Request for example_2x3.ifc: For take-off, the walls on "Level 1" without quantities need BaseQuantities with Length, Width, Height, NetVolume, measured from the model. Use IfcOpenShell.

First a look at what the model holds.

```python
import ifcopenshell
import ifcopenshell.util.element
import ifcopenshell.util.unit

model = ifcopenshell.open("example_2x3.ifc")
print(model.schema)
for unit_type in ("LENGTHUNIT", "AREAUNIT", "VOLUMEUNIT"):
    print(unit_type, ifcopenshell.util.unit.calculate_unit_scale(model, unit_type))
storey = next(s for s in model.by_type("IfcBuildingStorey") if s.Name == "Level 1")
walls = [e for e in ifcopenshell.util.element.get_decomposition(storey) if e.is_a("IfcWall")]
for e in sorted(walls, key=lambda e: e.id()):
    print(e.id(), e.is_a(), e.Name, list(ifcopenshell.util.element.get_psets(e, qtos_only=True)), sep=" | ")
```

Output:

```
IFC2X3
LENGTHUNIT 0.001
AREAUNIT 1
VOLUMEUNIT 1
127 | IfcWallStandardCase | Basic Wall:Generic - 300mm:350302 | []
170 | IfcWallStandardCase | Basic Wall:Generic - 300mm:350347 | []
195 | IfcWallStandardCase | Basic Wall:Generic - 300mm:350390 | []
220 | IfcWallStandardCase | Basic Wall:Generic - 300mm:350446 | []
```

```python
import ifcopenshell
import ifcopenshell.api.pset
import ifcopenshell.geom
import ifcopenshell.util.element
import ifcopenshell.util.shape
import ifcopenshell.util.unit

model = ifcopenshell.open("example_2x3.ifc")
unit_scale = ifcopenshell.util.unit.calculate_unit_scale(model)
volume_scale = ifcopenshell.util.unit.calculate_unit_scale(model, "VOLUMEUNIT")
settings = ifcopenshell.geom.settings()

storey = next(s for s in model.by_type("IfcBuildingStorey") if s.Name == "Level 1")
walls = [e for e in ifcopenshell.util.element.get_decomposition(storey) if e.is_a("IfcWall")]

for e in sorted(walls, key=lambda e: e.id()):
    if ifcopenshell.util.element.get_psets(e, qtos_only=True, should_inherit=False):
        continue
    # Geometry comes back in metres, in the element's own axes.
    shape = ifcopenshell.geom.create_shape(settings, e)
    values = {
        "Length": ifcopenshell.util.shape.get_x(shape.geometry) / unit_scale,
        "Width": ifcopenshell.util.shape.get_y(shape.geometry) / unit_scale,
        "Height": ifcopenshell.util.shape.get_z(shape.geometry) / unit_scale,
        "NetVolume": ifcopenshell.util.shape.get_volume(shape.geometry) / volume_scale,
    }
    qto = ifcopenshell.api.pset.add_qto(model, product=e, name="BaseQuantities")
    ifcopenshell.api.pset.edit_qto(model, qto=qto, properties=values)
    print(e.id(), {k: round(v, 3) for k, v in values.items()})

model.write("example_2x3_v2.ifc")
```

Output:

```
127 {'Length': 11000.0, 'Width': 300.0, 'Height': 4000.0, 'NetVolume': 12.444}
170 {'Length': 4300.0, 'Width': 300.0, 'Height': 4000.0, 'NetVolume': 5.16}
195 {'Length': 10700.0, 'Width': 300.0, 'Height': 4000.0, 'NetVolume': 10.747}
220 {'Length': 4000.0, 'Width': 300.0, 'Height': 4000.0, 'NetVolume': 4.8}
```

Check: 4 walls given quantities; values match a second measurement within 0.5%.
